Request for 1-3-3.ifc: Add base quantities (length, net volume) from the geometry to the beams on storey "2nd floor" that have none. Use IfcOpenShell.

First a look at what the model holds.

```python
import ifcopenshell
import ifcopenshell.util.element
import ifcopenshell.util.unit

model = ifcopenshell.open("1-3-3.ifc")
print(model.schema)
for unit_type in ("LENGTHUNIT", "AREAUNIT", "VOLUMEUNIT"):
    print(unit_type, ifcopenshell.util.unit.calculate_unit_scale(model, unit_type))
storey = next(s for s in model.by_type("IfcBuildingStorey") if s.Name == "2nd floor")
beams = [e for e in ifcopenshell.util.element.get_decomposition(storey) if e.is_a("IfcBeam")]
for e in sorted(beams, key=lambda e: e.id()):
    print(e.id(), e.is_a(), e.Name, list(ifcopenshell.util.element.get_psets(e, qtos_only=True)), sep=" | ")
```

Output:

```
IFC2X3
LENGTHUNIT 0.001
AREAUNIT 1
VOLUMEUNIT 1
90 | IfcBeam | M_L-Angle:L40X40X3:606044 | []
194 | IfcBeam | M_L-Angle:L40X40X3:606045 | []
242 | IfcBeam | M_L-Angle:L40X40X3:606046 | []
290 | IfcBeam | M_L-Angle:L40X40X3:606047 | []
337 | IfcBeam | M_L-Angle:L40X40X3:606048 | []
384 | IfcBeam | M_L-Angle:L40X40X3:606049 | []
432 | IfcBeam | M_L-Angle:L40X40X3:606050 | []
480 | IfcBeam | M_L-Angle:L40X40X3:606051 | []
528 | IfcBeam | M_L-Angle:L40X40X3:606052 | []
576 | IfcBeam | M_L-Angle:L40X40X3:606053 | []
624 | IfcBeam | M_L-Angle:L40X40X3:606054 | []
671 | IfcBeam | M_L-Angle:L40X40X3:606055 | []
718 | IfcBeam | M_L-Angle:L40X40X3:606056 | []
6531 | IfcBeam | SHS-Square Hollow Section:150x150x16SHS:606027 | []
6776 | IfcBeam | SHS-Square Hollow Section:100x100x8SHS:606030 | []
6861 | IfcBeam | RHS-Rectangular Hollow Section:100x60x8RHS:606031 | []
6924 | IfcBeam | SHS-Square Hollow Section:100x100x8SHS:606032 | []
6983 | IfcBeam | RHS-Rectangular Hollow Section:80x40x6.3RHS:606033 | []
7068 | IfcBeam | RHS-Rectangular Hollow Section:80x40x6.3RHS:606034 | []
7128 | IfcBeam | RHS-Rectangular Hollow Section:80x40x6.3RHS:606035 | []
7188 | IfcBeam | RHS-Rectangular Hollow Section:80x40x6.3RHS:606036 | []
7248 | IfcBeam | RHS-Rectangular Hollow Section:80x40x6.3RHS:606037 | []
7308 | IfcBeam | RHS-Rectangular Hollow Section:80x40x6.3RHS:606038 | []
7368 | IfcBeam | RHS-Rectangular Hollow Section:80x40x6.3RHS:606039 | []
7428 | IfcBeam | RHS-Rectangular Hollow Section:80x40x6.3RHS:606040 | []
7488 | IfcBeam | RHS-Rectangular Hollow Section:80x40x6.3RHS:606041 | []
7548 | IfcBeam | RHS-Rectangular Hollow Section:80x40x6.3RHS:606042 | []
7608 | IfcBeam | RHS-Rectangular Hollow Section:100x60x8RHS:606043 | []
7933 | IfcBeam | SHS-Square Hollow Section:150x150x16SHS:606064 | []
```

```python
import ifcopenshell
import ifcopenshell.api.pset
import ifcopenshell.geom
import ifcopenshell.util.element
import ifcopenshell.util.shape
import ifcopenshell.util.unit

model = ifcopenshell.open("1-3-3.ifc")
unit_scale = ifcopenshell.util.unit.calculate_unit_scale(model)
volume_scale = ifcopenshell.util.unit.calculate_unit_scale(model, "VOLUMEUNIT")
settings = ifcopenshell.geom.settings()

storey = next(s for s in model.by_type("IfcBuildingStorey") if s.Name == "2nd floor")
beams = [e for e in ifcopenshell.util.element.get_decomposition(storey) if e.is_a("IfcBeam")]

for e in sorted(beams, key=lambda e: e.id()):
    if ifcopenshell.util.element.get_psets(e, qtos_only=True, should_inherit=False):
        continue
    # Geometry comes back in metres, in the element's own axes.
    shape = ifcopenshell.geom.create_shape(settings, e)
    values = {
        "Length": ifcopenshell.util.shape.get_max_xyz(shape.geometry) / unit_scale,
        "NetVolume": ifcopenshell.util.shape.get_volume(shape.geometry) / volume_scale,
    }
    qto = ifcopenshell.api.pset.add_qto(model, product=e, name="BaseQuantities")
    ifcopenshell.api.pset.edit_qto(model, qto=qto, properties=values)
    print(e.id(), {k: round(v, 3) for k, v in values.items()})

model.write("1-3-3_edited.ifc")
```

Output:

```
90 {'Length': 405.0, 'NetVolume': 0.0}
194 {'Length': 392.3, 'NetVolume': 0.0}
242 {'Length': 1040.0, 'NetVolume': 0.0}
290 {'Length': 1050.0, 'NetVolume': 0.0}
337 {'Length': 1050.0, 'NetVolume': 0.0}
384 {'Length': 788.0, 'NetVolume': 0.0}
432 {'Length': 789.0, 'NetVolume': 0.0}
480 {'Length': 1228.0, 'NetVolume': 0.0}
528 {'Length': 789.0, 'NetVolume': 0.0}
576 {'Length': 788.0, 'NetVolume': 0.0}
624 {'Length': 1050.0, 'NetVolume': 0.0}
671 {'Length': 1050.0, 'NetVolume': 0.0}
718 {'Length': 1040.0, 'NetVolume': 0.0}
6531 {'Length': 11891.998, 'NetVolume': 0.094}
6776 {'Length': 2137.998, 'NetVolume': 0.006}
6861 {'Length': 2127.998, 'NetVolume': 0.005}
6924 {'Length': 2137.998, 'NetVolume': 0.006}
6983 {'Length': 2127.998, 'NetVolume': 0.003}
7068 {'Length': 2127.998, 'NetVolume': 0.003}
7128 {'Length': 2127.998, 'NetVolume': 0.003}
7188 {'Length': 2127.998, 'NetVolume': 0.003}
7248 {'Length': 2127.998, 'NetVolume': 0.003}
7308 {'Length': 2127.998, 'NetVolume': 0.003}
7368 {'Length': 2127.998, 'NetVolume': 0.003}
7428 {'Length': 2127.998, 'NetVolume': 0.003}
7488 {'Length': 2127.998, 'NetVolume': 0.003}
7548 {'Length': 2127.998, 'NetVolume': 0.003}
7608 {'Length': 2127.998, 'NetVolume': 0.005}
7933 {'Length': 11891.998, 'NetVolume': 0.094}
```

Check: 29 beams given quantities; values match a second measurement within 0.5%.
